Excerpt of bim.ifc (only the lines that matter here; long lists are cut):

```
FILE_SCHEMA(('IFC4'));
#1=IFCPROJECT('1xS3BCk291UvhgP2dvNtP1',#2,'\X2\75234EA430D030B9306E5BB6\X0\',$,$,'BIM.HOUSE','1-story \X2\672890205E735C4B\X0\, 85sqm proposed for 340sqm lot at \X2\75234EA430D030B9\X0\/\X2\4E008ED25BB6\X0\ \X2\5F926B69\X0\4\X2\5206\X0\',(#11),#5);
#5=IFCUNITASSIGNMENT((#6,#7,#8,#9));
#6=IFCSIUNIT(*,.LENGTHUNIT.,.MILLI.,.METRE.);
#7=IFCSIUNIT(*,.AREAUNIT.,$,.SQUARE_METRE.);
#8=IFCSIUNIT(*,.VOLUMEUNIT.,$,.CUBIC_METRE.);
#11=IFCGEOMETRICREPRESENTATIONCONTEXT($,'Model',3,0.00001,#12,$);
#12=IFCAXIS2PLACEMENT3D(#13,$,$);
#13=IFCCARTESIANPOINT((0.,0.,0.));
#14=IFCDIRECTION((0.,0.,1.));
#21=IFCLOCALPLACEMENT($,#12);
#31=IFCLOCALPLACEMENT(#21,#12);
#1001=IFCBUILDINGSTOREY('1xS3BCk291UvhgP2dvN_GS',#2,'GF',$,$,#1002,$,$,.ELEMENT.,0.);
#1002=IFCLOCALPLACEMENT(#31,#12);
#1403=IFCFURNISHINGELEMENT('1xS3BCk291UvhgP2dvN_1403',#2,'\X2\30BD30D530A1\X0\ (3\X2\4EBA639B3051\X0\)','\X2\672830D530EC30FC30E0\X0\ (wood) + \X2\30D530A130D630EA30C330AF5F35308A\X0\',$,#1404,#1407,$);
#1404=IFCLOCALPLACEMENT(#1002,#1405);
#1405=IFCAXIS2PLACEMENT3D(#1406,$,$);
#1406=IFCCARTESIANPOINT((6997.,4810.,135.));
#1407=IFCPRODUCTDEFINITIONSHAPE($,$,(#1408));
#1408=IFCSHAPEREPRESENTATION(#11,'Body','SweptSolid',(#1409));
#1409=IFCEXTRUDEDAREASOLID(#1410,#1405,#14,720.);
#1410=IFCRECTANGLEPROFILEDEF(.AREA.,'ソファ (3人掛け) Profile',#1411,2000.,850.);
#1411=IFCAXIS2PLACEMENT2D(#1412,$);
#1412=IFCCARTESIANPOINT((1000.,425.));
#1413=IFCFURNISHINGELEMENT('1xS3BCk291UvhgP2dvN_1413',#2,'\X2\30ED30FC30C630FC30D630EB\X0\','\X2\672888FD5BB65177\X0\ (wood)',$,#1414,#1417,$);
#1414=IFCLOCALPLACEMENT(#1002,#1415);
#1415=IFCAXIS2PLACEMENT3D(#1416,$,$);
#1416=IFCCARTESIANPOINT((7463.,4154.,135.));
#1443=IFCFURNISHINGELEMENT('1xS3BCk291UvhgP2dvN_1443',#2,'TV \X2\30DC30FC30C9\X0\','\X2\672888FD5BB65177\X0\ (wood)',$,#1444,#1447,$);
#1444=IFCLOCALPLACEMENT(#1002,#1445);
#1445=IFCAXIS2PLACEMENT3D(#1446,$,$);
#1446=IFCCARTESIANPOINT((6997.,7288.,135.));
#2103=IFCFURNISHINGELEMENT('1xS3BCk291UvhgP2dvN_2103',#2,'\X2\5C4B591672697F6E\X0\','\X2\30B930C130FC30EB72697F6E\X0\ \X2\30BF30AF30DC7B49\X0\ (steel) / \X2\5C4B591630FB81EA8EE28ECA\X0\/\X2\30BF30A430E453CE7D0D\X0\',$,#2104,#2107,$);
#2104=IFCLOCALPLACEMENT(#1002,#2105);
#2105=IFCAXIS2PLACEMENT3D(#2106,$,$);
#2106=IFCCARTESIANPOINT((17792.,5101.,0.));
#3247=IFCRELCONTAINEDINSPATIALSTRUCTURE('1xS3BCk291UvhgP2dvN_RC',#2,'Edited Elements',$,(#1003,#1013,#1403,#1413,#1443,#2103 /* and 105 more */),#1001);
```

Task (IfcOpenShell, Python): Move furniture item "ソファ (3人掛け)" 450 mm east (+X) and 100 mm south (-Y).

```python
import ifcopenshell
import ifcopenshell.api.geometry
import ifcopenshell.util.placement
import ifcopenshell.util.unit

model = ifcopenshell.open("bim.ifc")
unit_scale = ifcopenshell.util.unit.calculate_unit_scale(model)

item = model.by_guid("1xS3BCk291UvhgP2dvN_1403")
matrix = ifcopenshell.util.placement.get_local_placement(item.ObjectPlacement)
matrix[0, 3] += 0.45 / unit_scale
matrix[1, 3] -= 0.1 / unit_scale
ifcopenshell.api.geometry.edit_object_placement(model, product=item, matrix=matrix, is_si=False)

print(ifcopenshell.util.placement.get_local_placement(item.ObjectPlacement).round(3) + 0.0)

model.write("bim_rev.ifc")
```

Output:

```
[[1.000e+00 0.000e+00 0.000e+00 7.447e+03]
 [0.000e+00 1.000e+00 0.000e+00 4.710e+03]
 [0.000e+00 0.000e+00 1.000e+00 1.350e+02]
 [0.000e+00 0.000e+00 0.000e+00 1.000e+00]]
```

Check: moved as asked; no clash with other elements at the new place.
